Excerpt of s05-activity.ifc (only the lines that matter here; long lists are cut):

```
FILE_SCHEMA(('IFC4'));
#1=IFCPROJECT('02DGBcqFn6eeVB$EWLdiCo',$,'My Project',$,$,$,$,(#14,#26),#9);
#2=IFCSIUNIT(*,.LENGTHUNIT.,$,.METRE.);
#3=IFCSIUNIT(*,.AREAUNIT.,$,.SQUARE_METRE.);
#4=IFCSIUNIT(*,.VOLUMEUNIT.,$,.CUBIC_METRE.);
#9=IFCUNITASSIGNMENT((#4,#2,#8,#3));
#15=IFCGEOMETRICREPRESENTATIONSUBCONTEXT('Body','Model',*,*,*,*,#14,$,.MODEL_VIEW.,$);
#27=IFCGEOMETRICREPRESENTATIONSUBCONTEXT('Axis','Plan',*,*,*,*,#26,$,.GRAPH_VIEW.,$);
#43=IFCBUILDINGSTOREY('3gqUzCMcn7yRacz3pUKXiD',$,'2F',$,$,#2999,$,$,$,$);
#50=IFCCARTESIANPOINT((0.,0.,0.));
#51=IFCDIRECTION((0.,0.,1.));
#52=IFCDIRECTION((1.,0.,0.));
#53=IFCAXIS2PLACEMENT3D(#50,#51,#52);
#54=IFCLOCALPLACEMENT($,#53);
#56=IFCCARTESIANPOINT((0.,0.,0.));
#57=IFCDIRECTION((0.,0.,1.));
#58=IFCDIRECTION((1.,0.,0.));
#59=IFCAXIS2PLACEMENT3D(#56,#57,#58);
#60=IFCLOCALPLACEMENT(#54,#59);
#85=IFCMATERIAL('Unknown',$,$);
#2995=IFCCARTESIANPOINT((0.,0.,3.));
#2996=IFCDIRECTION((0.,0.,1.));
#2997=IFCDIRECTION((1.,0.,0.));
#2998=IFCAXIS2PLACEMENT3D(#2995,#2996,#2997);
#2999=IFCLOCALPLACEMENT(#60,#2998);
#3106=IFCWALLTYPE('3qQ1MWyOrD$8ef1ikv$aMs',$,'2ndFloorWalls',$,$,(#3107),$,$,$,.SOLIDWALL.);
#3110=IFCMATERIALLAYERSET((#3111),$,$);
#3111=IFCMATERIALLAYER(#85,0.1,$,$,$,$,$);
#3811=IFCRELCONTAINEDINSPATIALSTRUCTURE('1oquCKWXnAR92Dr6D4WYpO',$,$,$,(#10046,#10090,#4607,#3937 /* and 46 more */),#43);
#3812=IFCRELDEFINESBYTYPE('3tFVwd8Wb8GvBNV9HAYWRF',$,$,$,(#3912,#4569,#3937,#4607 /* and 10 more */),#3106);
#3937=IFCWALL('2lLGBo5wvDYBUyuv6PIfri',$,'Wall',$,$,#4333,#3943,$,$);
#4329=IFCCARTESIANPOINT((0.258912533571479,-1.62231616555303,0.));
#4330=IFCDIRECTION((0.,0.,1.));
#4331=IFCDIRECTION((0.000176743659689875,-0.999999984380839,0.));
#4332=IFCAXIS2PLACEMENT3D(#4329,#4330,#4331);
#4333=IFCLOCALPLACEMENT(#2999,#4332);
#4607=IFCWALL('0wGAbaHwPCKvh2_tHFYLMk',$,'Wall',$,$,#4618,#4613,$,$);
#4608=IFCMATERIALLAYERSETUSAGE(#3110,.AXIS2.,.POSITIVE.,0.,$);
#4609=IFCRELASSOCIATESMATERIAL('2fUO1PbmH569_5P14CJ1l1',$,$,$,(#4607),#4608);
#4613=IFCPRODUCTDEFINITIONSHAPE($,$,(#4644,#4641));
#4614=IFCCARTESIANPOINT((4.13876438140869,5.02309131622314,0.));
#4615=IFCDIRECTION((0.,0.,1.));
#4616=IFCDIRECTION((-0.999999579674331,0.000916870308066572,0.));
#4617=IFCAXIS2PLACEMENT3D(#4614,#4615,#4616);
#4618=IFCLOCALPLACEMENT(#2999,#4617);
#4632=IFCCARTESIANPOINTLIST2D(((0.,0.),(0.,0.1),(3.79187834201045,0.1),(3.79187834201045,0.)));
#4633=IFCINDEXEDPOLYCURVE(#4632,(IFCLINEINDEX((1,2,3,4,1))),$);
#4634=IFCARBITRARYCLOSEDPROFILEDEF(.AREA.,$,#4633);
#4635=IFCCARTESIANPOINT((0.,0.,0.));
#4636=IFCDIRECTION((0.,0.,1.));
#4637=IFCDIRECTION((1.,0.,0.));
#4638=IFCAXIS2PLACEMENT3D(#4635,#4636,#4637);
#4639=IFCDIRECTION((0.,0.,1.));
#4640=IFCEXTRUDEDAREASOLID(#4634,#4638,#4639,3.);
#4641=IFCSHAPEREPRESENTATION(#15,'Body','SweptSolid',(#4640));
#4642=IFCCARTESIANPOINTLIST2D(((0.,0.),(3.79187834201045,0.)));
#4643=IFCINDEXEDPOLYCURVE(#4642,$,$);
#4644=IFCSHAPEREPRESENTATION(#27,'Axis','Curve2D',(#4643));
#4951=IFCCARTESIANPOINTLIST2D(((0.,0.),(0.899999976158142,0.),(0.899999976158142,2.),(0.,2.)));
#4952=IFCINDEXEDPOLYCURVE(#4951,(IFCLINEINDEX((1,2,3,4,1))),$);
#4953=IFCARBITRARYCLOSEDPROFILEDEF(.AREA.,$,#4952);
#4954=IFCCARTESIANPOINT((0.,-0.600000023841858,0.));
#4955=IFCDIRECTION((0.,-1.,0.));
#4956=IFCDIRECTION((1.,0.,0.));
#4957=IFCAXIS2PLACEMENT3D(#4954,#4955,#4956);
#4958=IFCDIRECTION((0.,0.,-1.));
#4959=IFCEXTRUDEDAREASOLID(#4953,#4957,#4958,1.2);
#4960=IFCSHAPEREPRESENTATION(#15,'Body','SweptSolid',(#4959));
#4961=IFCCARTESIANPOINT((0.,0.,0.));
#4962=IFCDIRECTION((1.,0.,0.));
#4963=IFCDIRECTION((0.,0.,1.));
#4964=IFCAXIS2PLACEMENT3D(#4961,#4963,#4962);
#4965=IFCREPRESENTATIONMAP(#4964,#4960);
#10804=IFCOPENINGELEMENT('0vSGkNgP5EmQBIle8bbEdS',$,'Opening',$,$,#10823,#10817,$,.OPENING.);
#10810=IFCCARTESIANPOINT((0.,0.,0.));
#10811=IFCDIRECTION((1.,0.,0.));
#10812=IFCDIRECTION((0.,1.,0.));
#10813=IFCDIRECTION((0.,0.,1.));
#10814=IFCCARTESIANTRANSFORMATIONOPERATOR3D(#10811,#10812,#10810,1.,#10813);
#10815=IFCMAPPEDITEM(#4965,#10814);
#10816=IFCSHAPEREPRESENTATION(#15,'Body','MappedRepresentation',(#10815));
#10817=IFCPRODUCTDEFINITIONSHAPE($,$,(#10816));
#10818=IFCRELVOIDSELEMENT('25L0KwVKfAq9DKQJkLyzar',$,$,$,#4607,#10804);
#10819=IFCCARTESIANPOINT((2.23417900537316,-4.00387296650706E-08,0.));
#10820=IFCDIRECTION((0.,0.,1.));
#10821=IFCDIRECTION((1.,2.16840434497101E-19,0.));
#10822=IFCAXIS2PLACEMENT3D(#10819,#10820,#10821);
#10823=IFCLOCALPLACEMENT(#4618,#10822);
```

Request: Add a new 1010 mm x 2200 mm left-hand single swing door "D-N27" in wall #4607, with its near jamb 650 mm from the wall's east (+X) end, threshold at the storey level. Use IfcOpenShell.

```python
import numpy as np
import ifcopenshell
import ifcopenshell.api.feature
import ifcopenshell.api.geometry
import ifcopenshell.api.root
import ifcopenshell.api.spatial
import ifcopenshell.geom
import ifcopenshell.util.element
import ifcopenshell.util.placement
import ifcopenshell.util.representation
import ifcopenshell.util.shape
import ifcopenshell.util.unit

model = ifcopenshell.open("s05-activity.ifc")
unit_scale = ifcopenshell.util.unit.calculate_unit_scale(model)
settings = ifcopenshell.geom.settings()


def volume(element):
    """Net volume in cubic metres, openings subtracted."""
    shape = ifcopenshell.geom.create_shape(settings, element)
    return ifcopenshell.util.shape.get_volume(shape.geometry)


wall = model.by_guid("0wGAbaHwPCKvh2_tHFYLMk")
storey = ifcopenshell.util.element.get_container(wall, ifc_class="IfcBuildingStorey")
context = ifcopenshell.util.representation.get_context(model, "Model", "Body", "MODEL_VIEW")
before = volume(wall)

width, height, from_end, sill = 1.01, 2.2, 0.65, 0.0  # metres

# The wall runs along its own X axis, and the end named is its -X end.
wall_shape = ifcopenshell.geom.create_shape(settings, wall)
x, y, z = ifcopenshell.util.shape.get_vertices(wall_shape.geometry).T
start = x.min() + from_end
face, thickness = float(y.min()), float(y.max() - y.min())
wall_matrix = ifcopenshell.util.placement.get_local_placement(wall.ObjectPlacement)
level = ifcopenshell.util.placement.get_local_placement(storey.ObjectPlacement)[2, 3]


def in_wall(x, y):
    """Placement at x, y metres in the wall's axes, at sill height."""
    matrix = wall_matrix.copy()
    matrix[:, 3] = wall_matrix @ np.array([x / unit_scale, y / unit_scale, 0.0, 1.0])
    matrix[2, 3] = level + sill / unit_scale
    return matrix


# Opening: a box that overshoots both wall faces by 50 mm.
opening = ifcopenshell.api.root.create_entity(model, ifc_class="IfcOpeningElement", predefined_type="OPENING")
box = ifcopenshell.api.geometry.add_wall_representation(
    model, context=context, length=width, height=height, thickness=thickness + 0.1
)
ifcopenshell.api.geometry.assign_representation(model, product=opening, representation=box)
ifcopenshell.api.geometry.edit_object_placement(model, product=opening, matrix=in_wall(start, face - 0.05), is_si=False)
ifcopenshell.api.feature.add_feature(model, feature=opening, element=wall)

door = ifcopenshell.api.root.create_entity(model, ifc_class="IfcDoor", name="D-N27", predefined_type="DOOR")
door.OverallWidth, door.OverallHeight = width / unit_scale, height / unit_scale
door.OperationType = "SINGLE_SWING_LEFT"
body = ifcopenshell.api.geometry.add_door_representation(
    model,
    context=context,
    overall_width=door.OverallWidth,
    overall_height=door.OverallHeight,
    operation_type="SINGLE_SWING_LEFT",
    lining_properties={"LiningDepth": thickness / unit_scale, "ThresholdDepth": thickness / unit_scale},
)
ifcopenshell.api.geometry.assign_representation(model, product=door, representation=body)
ifcopenshell.api.spatial.assign_container(model, products=[door], relating_structure=storey)
ifcopenshell.api.feature.add_filling(model, opening=opening, element=door)

# The lining spans the wall, so the door starts at the wall face.
ifcopenshell.api.geometry.edit_object_placement(model, product=door, matrix=in_wall(start, face), is_si=False)

after = volume(wall)

print(f"wall volume {before:.3f} -> {after:.3f} m3")

model.write("s05-activity-out.ifc")
```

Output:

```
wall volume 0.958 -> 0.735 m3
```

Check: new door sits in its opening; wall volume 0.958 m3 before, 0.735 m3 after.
